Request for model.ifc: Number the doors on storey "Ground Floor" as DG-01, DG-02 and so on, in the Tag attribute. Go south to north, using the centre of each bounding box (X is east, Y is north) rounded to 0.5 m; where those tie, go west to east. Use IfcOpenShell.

First a look at what the model holds.

```python
import ifcopenshell
import ifcopenshell.util.element
import ifcopenshell.util.placement

model = ifcopenshell.open("model.ifc")
print(model.schema)
storey = next(s for s in model.by_type("IfcBuildingStorey") if s.Name == "Ground Floor")
doors = [e for e in ifcopenshell.util.element.get_decomposition(storey) if e.is_a("IfcDoor")]
for e in sorted(doors, key=lambda e: e.id()):
    origin = ifcopenshell.util.placement.get_local_placement(e.ObjectPlacement)[:3, 3]
    print(e.id(), e.Tag, e.Name, origin.round(2) + 0.0, sep=" | ")
```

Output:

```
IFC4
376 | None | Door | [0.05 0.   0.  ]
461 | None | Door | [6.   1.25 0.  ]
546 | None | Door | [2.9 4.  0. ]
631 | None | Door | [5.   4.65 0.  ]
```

```python
import ifcopenshell
import ifcopenshell.geom
import ifcopenshell.util.element
import ifcopenshell.util.shape

model = ifcopenshell.open("model.ifc")
settings = ifcopenshell.geom.settings()
settings.set("use-world-coords", True)


def centre(element):
    shape = ifcopenshell.geom.create_shape(settings, element)
    return ifcopenshell.util.shape.get_bbox_centroid(shape.geometry)


storey = next(s for s in model.by_type("IfcBuildingStorey") if s.Name == "Ground Floor")
doors = [e for e in ifcopenshell.util.element.get_decomposition(storey) if e.is_a("IfcDoor")]

# Insertion points can sit at a corner or the storey origin, so sort by the geometry (in metres).
centres = {e: centre(e) for e in doors}
doors.sort(key=lambda e: (round(centres[e][1] / 0.5), centres[e][0]))

for i, e in enumerate(doors, start=1):
    number = f"DG-{i:02d}"
    e.Tag = number
    print(e.id(), number)

model.write("model_edited.ifc")
```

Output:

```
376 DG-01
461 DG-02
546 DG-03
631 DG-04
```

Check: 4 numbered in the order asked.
